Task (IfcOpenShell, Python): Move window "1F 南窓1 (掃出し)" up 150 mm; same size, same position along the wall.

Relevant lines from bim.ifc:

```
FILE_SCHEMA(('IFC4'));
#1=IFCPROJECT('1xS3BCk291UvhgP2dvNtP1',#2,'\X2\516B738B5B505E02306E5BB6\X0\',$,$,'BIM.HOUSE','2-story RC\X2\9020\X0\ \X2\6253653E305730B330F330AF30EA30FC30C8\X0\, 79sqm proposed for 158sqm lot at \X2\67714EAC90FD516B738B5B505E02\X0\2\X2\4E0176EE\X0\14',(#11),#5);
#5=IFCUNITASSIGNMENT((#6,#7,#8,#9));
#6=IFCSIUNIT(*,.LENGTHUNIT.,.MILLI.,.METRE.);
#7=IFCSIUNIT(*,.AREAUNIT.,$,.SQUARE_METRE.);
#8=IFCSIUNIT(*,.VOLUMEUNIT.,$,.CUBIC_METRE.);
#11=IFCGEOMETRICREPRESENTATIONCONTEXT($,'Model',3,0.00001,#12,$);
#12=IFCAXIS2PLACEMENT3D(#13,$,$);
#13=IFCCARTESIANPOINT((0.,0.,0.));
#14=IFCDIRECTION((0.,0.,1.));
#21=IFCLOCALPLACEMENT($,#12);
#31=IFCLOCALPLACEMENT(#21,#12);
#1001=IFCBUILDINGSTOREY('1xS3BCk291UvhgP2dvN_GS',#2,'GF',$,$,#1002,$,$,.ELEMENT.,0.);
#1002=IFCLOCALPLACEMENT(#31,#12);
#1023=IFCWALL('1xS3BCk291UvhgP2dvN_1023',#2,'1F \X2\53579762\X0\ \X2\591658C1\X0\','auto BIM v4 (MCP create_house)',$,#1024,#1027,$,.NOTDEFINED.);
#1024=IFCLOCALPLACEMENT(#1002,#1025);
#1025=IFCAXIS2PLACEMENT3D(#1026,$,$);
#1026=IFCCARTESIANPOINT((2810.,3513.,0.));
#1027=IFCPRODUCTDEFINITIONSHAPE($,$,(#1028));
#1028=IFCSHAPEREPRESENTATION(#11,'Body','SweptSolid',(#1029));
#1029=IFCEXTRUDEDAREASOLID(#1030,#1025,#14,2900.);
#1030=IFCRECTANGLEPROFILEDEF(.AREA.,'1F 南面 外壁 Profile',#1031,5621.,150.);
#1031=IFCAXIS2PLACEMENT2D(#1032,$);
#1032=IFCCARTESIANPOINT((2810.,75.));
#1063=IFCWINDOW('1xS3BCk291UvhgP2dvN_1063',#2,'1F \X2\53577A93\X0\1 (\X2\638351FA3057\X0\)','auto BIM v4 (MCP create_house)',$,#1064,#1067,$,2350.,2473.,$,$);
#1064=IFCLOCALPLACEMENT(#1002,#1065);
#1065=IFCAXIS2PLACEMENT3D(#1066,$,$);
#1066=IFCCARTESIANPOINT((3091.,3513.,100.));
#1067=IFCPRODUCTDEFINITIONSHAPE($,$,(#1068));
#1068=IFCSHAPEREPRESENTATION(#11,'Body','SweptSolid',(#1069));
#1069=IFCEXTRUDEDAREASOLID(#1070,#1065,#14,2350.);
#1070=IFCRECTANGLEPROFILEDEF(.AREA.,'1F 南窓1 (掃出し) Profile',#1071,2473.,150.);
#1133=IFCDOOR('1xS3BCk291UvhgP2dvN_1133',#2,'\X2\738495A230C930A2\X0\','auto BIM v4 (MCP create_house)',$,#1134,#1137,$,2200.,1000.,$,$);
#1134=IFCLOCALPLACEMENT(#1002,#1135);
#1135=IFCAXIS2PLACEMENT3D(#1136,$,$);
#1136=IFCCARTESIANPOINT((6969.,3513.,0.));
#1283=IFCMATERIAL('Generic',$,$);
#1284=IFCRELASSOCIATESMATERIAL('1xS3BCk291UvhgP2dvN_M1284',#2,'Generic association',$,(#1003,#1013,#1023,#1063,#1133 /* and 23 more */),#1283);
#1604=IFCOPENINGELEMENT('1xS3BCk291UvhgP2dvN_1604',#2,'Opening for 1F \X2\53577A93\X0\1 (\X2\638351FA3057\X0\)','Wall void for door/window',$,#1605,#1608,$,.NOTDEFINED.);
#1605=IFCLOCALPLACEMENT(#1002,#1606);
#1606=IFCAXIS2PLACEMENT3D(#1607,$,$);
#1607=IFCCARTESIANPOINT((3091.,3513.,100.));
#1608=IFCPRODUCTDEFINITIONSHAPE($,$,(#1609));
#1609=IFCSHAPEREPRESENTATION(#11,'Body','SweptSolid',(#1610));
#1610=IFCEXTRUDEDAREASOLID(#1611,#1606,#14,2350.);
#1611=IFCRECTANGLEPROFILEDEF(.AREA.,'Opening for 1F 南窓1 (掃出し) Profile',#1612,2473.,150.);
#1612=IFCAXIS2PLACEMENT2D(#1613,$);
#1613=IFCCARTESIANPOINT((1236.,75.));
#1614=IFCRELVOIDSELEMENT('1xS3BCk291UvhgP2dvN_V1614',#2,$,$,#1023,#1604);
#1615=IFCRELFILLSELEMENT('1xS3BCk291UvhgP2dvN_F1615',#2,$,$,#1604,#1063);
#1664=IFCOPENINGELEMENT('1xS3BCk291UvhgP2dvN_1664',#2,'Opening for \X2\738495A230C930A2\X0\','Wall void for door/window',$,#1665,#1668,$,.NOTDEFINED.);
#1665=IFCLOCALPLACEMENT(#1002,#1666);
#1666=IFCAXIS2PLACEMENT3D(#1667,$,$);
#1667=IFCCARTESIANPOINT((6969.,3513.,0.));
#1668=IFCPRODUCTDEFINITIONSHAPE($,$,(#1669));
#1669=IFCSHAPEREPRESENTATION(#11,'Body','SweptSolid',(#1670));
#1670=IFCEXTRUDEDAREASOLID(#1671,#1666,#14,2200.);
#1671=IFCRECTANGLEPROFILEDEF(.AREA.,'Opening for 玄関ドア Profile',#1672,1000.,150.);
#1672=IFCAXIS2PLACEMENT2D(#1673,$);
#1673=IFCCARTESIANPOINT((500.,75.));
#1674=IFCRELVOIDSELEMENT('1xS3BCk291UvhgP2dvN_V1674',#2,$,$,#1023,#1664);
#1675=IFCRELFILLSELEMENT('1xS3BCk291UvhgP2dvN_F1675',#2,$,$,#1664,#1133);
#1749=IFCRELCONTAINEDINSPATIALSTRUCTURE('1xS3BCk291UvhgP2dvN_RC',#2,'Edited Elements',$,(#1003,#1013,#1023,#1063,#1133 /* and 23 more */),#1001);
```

```python
import numpy as np
import ifcopenshell
import ifcopenshell.api.geometry
import ifcopenshell.util.placement
import ifcopenshell.util.unit

model = ifcopenshell.open("bim.ifc")
unit_scale = ifcopenshell.util.unit.calculate_unit_scale(model)

window = model.by_guid("1xS3BCk291UvhgP2dvN_1063")
opening = window.FillsVoids[0].RelatingOpeningElement
dz = 150.0

shift = np.array([0.0, 0.0, dz])
# The window is not placed relative to its opening, so move both.
for product in (opening, window):
    matrix = ifcopenshell.util.placement.get_local_placement(product.ObjectPlacement)
    matrix[:3, 3] += shift
    ifcopenshell.api.geometry.edit_object_placement(model, product=product, matrix=matrix, is_si=False)

print(f"moved by {dz * unit_scale:+.3f} m")

model.write("bim_v2.ifc")
```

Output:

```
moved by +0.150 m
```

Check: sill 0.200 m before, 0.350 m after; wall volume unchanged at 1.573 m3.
